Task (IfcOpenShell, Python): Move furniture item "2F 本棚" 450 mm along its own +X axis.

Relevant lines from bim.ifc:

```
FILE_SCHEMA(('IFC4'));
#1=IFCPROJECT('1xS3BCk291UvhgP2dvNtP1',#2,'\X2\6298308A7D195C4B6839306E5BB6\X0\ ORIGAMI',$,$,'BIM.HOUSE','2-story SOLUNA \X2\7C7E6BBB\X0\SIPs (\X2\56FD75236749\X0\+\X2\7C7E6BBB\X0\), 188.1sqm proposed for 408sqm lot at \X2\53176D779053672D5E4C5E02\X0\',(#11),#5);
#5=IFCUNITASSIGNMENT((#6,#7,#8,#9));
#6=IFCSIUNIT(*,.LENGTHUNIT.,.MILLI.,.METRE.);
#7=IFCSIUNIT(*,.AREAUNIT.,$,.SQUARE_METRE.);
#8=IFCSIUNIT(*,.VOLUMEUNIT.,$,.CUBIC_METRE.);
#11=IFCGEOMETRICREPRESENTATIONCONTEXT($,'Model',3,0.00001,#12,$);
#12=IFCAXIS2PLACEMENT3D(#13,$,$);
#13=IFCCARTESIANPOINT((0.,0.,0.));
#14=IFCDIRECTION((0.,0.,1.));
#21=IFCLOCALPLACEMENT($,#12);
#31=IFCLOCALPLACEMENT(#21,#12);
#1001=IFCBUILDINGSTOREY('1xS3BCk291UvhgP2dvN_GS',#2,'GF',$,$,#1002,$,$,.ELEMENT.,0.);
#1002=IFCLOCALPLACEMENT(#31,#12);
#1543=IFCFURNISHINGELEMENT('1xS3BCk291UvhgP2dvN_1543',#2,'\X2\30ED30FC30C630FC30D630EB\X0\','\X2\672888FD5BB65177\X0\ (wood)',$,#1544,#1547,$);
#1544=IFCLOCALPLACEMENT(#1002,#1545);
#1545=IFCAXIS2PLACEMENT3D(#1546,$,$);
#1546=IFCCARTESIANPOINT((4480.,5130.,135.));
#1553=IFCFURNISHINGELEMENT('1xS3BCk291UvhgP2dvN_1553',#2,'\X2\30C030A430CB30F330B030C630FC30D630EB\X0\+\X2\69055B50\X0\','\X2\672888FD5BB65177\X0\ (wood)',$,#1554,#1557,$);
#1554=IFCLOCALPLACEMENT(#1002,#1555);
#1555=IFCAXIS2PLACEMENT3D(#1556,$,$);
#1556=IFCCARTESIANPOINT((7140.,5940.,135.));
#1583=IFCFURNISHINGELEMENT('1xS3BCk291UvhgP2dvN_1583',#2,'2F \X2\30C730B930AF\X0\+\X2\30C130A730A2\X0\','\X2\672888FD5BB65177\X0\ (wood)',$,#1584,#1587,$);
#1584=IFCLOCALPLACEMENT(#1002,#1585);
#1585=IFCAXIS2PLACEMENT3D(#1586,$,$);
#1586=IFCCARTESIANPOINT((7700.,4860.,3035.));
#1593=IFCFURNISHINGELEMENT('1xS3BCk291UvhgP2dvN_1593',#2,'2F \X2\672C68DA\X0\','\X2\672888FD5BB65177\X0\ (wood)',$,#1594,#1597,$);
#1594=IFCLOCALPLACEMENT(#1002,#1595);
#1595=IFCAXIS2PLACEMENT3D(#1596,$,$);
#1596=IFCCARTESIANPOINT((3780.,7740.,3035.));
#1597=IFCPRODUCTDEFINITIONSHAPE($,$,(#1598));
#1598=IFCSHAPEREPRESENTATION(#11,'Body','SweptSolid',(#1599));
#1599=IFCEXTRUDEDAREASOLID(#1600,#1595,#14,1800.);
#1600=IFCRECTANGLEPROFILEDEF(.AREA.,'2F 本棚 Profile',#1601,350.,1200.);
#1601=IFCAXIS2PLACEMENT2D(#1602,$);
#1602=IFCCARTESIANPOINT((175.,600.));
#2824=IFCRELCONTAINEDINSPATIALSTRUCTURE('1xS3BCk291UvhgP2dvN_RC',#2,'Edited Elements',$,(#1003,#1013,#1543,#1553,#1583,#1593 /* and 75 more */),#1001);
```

```python
import ifcopenshell
import ifcopenshell.api.geometry
import ifcopenshell.util.placement

model = ifcopenshell.open("bim.ifc")

item = model.by_id(1593)
matrix = ifcopenshell.util.placement.get_local_placement(item.ObjectPlacement)
matrix[:3, 3] += matrix[:3, 0] * 450.0
ifcopenshell.api.geometry.edit_object_placement(model, product=item, matrix=matrix, is_si=False)

print(ifcopenshell.util.placement.get_local_placement(item.ObjectPlacement).round(3) + 0.0)

model.write("bim_rev.ifc")
```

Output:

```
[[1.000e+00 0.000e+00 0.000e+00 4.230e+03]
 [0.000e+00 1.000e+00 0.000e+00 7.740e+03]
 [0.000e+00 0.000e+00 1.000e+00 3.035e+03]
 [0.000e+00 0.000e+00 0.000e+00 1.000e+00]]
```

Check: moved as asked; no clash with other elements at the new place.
